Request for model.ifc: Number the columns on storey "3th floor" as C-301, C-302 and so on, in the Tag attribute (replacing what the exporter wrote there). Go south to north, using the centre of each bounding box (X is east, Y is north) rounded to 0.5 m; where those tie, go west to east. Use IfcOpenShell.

First a look at what the model holds.

```python
import ifcopenshell
import ifcopenshell.util.element
import ifcopenshell.util.placement

model = ifcopenshell.open("model.ifc")
print(model.schema)
storey = next(s for s in model.by_type("IfcBuildingStorey") if s.Name == "3th floor")
columns = [e for e in ifcopenshell.util.element.get_decomposition(storey) if e.is_a("IfcColumn")]
for e in sorted(columns, key=lambda e: e.id()):
    origin = ifcopenshell.util.placement.get_local_placement(e.ObjectPlacement)[:3, 3]
    print(e.id(), e.Tag, e.Name, origin.round(2) + 0.0, sep=" | ")
```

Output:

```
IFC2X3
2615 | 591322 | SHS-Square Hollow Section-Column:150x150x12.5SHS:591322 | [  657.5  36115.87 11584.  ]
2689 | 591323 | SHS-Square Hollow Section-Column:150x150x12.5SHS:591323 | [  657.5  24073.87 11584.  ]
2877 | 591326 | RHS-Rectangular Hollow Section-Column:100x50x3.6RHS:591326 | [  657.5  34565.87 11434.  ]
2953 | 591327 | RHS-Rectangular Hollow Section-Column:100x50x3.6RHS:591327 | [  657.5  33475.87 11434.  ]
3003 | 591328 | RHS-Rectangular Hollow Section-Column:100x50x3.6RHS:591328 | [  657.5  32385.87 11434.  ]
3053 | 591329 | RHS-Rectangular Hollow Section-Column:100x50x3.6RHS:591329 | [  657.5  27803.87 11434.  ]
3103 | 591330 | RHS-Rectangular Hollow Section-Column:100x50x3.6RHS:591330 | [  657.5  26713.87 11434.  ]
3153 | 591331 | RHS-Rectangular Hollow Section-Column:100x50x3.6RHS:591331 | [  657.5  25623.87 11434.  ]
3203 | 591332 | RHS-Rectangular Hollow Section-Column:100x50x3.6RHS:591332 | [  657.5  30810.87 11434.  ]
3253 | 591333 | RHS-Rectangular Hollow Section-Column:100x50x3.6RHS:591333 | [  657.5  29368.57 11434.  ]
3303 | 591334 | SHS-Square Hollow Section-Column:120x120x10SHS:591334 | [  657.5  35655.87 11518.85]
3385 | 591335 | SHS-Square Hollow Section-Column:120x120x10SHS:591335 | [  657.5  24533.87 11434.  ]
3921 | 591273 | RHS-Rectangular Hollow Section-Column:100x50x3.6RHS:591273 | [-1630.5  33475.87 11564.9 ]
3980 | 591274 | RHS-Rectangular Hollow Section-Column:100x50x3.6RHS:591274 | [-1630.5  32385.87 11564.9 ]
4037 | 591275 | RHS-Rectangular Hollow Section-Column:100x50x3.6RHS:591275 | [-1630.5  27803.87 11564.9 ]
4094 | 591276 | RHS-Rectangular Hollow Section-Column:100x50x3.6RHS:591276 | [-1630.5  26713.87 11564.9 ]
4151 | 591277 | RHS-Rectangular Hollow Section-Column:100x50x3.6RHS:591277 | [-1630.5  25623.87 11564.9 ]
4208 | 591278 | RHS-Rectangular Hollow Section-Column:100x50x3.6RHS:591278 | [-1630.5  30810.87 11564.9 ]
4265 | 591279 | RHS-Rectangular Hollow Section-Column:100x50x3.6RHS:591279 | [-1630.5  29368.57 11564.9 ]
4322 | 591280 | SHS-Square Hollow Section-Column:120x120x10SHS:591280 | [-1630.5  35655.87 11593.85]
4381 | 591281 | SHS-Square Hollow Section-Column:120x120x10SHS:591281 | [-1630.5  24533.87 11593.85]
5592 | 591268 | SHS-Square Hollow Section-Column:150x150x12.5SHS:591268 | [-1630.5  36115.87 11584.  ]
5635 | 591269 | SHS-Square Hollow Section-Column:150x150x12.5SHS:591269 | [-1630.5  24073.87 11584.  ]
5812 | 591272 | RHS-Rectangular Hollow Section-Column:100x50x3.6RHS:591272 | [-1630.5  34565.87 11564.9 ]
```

```python
import ifcopenshell
import ifcopenshell.geom
import ifcopenshell.util.element
import ifcopenshell.util.shape

model = ifcopenshell.open("model.ifc")
settings = ifcopenshell.geom.settings()
settings.set("use-world-coords", True)


def centre(element):
    shape = ifcopenshell.geom.create_shape(settings, element)
    return ifcopenshell.util.shape.get_bbox_centroid(shape.geometry)


storey = next(s for s in model.by_type("IfcBuildingStorey") if s.Name == "3th floor")
columns = [e for e in ifcopenshell.util.element.get_decomposition(storey) if e.is_a("IfcColumn")]

# Insertion points can sit at a corner or the storey origin, so sort by the geometry (in metres).
centres = {e: centre(e) for e in columns}
columns.sort(key=lambda e: (round(centres[e][1] / 0.5), centres[e][0]))

for i, e in enumerate(columns, start=1):
    number = f"C-3{i:02d}"
    e.Tag = number
    print(e.id(), number)

model.write("model_rev.ifc")
```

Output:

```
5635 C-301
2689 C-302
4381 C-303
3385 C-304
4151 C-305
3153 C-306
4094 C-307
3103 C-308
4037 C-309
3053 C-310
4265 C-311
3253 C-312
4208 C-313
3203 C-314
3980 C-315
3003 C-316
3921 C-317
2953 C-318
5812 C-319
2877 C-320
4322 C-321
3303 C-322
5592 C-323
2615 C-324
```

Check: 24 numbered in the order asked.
